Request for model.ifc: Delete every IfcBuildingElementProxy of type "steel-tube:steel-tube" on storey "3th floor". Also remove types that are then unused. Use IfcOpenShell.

First a look at what the model holds.

```python
import ifcopenshell
import ifcopenshell.util.element

model = ifcopenshell.open("model.ifc")
print(model.schema)
storey = next(s for s in model.by_type("IfcBuildingStorey") if s.Name == "3th floor")
proxies = [e for e in ifcopenshell.util.element.get_decomposition(storey) if e.is_a("IfcBuildingElementProxy")]
seen = {}
for e in proxies:
    element_type = ifcopenshell.util.element.get_type(e)
    name = element_type.Name if element_type not in (None, e) else None
    seen[name] = seen.get(name, 0) + 1
for name, count in sorted(seen.items(), key=str):
    print(count, "x", name)
```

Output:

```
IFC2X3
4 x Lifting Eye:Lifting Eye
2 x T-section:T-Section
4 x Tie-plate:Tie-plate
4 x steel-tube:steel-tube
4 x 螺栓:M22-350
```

```python
import ifcopenshell
import ifcopenshell.api.root
import ifcopenshell.util.element

model = ifcopenshell.open("model.ifc")

storey = next(s for s in model.by_type("IfcBuildingStorey") if s.Name == "3th floor")
proxies = [e for e in ifcopenshell.util.element.get_decomposition(storey) if e.is_a("IfcBuildingElementProxy")]
targets = [e for e in proxies if (t := ifcopenshell.util.element.get_type(e)) not in (None, e) and t.Name == "steel-tube:steel-tube"]
types = {ifcopenshell.util.element.get_type(e) for e in targets} - {None, *targets}

for e in targets:
    ifcopenshell.api.root.remove_product(model, product=e)
print(len(targets), "removed")

unused = [t for t in types if not ifcopenshell.util.element.get_types(t)]
for t in unused:
    ifcopenshell.api.root.remove_product(model, product=t)
print(len(unused), "unused types removed")

model.write("model_edited.ifc")
```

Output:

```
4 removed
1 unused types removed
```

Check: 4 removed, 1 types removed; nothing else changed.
